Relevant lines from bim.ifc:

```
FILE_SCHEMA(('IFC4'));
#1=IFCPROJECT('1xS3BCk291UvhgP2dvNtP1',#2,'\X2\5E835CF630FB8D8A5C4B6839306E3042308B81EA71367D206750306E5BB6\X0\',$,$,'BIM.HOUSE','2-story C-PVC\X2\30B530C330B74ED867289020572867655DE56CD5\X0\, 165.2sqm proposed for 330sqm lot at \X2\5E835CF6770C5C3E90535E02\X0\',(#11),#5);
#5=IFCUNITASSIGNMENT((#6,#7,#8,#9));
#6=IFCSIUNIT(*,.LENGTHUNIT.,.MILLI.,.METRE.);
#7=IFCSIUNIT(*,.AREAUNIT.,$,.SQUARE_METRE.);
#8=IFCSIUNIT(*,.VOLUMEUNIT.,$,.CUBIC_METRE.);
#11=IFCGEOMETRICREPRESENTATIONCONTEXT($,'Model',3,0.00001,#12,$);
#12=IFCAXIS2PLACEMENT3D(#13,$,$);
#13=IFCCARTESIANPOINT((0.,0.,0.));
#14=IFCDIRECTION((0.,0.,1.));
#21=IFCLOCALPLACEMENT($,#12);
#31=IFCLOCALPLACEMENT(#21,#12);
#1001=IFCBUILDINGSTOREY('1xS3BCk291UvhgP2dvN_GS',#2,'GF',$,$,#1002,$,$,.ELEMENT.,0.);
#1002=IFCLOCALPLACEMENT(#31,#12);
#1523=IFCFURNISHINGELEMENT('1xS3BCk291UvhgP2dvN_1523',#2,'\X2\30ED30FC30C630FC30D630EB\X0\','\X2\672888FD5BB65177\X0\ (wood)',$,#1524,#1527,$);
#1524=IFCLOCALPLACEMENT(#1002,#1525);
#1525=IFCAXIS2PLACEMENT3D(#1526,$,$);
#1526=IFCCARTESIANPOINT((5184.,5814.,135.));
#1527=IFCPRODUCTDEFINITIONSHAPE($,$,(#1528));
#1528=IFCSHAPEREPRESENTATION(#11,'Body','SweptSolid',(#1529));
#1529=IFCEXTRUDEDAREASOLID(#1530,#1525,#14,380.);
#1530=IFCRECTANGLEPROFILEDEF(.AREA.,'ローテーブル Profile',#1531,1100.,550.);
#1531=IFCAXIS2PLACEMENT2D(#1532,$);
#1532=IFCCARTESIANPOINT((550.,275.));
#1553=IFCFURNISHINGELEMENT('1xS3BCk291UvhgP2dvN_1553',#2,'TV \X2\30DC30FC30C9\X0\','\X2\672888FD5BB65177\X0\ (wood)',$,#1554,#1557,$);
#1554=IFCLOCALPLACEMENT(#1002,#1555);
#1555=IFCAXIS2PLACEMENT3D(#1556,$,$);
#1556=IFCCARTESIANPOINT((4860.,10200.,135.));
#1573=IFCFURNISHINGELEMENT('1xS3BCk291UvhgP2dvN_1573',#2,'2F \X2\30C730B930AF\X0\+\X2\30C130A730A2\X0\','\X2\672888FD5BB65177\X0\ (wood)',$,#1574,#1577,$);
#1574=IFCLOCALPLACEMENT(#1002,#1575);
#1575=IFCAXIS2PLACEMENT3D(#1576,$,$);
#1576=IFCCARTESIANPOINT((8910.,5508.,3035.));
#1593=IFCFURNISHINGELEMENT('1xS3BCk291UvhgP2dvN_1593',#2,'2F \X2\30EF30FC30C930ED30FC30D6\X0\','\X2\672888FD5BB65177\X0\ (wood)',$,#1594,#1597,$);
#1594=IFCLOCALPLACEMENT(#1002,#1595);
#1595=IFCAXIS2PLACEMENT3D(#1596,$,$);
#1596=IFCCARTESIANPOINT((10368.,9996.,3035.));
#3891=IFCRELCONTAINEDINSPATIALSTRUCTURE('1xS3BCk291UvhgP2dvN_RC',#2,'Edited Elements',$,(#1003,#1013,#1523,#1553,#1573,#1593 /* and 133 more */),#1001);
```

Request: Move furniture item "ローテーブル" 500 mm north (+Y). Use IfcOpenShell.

```python
import ifcopenshell
import ifcopenshell.api.geometry
import ifcopenshell.util.placement
import ifcopenshell.util.unit

model = ifcopenshell.open("bim.ifc")
unit_scale = ifcopenshell.util.unit.calculate_unit_scale(model)

item = model.by_guid("1xS3BCk291UvhgP2dvN_1523")
matrix = ifcopenshell.util.placement.get_local_placement(item.ObjectPlacement)
matrix[1, 3] += 0.5 / unit_scale
ifcopenshell.api.geometry.edit_object_placement(model, product=item, matrix=matrix, is_si=False)

print(ifcopenshell.util.placement.get_local_placement(item.ObjectPlacement).round(3) + 0.0)

model.write("bim-out.ifc")
```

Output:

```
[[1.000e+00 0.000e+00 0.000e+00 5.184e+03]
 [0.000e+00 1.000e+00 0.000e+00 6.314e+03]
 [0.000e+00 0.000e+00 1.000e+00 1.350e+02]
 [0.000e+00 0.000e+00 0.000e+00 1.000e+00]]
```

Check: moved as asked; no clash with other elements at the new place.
